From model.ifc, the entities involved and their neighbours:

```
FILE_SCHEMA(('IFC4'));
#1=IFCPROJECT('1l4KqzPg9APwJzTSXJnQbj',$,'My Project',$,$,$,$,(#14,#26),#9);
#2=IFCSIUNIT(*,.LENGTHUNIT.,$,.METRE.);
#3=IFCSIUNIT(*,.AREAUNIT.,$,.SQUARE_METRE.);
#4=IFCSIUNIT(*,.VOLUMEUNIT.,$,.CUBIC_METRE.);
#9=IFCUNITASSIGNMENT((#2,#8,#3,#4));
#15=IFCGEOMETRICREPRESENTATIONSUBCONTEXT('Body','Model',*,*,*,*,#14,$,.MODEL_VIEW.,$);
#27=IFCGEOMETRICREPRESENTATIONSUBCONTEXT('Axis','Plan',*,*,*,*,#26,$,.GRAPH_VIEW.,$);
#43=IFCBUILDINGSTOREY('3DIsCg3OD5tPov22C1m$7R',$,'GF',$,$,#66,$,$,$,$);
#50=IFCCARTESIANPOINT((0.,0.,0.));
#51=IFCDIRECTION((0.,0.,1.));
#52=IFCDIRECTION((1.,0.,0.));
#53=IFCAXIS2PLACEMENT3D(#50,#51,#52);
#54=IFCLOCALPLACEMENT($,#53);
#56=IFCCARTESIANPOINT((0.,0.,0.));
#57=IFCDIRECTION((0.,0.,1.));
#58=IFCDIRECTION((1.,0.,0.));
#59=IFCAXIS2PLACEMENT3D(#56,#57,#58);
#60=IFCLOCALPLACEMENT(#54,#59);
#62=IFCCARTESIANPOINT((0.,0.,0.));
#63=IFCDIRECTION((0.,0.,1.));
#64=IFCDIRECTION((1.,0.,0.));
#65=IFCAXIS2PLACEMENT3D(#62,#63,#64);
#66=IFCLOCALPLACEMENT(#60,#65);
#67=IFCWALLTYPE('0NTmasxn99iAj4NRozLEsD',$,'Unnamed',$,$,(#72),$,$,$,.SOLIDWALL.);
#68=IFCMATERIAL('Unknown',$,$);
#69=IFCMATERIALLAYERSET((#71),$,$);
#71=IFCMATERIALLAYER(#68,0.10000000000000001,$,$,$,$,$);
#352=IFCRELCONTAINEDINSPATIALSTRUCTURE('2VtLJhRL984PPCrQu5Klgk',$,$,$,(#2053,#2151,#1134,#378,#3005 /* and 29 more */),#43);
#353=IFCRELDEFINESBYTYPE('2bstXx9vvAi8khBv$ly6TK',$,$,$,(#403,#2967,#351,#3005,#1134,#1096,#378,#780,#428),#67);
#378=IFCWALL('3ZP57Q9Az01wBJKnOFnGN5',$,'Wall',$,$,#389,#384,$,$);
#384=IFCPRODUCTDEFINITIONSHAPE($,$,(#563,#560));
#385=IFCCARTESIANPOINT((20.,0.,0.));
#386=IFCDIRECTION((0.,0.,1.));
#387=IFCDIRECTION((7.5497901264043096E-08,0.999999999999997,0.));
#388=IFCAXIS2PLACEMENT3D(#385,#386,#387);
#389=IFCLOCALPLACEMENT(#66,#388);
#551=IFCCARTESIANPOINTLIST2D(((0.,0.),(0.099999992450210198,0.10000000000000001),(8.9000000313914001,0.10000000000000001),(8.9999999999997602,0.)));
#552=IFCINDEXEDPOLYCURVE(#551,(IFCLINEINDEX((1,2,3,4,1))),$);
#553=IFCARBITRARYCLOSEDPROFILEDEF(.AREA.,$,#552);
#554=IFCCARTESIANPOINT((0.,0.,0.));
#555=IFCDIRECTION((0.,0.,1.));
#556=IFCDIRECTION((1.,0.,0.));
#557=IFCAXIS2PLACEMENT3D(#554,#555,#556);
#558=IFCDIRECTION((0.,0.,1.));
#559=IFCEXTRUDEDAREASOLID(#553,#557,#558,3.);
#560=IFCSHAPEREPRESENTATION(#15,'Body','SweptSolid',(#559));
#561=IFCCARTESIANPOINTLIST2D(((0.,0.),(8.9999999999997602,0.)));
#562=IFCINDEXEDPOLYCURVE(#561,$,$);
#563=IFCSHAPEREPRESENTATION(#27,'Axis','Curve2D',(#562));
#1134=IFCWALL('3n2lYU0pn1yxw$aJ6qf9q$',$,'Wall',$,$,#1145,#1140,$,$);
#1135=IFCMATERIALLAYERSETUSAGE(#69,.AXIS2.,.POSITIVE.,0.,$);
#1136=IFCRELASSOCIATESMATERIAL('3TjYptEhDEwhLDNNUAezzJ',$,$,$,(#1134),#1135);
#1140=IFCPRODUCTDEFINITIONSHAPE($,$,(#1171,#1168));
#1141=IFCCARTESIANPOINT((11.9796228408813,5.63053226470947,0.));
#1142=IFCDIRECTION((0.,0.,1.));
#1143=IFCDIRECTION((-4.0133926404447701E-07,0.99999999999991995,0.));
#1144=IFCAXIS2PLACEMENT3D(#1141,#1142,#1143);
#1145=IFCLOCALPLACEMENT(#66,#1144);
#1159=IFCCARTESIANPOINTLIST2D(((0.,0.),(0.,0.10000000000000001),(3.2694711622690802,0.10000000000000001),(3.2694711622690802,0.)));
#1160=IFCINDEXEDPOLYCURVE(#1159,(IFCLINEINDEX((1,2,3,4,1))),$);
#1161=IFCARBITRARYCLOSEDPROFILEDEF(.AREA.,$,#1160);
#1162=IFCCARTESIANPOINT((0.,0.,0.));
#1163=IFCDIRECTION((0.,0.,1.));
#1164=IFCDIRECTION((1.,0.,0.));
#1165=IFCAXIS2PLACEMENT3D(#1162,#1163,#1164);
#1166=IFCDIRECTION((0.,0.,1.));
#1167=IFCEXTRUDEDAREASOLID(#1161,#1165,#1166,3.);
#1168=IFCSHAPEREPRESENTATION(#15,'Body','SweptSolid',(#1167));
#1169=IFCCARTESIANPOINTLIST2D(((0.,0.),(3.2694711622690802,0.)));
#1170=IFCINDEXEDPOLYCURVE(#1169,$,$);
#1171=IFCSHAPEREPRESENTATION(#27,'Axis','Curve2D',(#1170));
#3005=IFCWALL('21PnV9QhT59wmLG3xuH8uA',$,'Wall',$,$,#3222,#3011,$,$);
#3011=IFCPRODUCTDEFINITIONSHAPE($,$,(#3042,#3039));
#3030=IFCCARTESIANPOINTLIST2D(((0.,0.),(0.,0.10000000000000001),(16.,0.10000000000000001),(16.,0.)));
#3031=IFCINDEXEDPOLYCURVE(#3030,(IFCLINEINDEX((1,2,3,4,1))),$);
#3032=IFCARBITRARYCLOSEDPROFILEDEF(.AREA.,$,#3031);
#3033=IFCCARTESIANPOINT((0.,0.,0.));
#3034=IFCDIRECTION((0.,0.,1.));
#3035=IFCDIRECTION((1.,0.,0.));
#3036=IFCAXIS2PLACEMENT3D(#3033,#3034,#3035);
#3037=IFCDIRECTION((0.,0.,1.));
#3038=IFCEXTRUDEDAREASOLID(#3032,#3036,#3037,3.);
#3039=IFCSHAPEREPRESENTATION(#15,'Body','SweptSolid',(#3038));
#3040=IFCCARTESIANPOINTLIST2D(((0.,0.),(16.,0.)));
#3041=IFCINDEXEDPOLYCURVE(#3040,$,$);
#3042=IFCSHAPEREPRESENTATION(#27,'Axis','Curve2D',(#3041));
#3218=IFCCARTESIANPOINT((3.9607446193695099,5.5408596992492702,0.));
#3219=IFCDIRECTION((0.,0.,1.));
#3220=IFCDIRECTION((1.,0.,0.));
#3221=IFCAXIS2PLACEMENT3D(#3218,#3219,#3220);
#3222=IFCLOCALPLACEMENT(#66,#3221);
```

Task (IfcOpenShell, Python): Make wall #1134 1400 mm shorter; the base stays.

```python
import ifcopenshell
import ifcopenshell.geom
import ifcopenshell.util.representation
import ifcopenshell.util.shape
import ifcopenshell.util.unit

model = ifcopenshell.open("model.ifc")
unit_scale = ifcopenshell.util.unit.calculate_unit_scale(model)
settings = ifcopenshell.geom.settings()


def volume(element):
    """Net volume in cubic metres, openings subtracted."""
    shape = ifcopenshell.geom.create_shape(settings, element)
    return ifcopenshell.util.shape.get_volume(shape.geometry)


wall = model.by_id(1134)
before = volume(wall)

body = ifcopenshell.util.representation.get_representation(wall, "Model", "Body")
solid = body.Items[0]
old_height = solid.Depth
solid.Depth -= 1.4 / unit_scale
after = volume(wall)

print(f"height {old_height:g} -> {solid.Depth:g}, volume {before:.3f} -> {after:.3f} m3")

model.write("model_v2.ifc")
```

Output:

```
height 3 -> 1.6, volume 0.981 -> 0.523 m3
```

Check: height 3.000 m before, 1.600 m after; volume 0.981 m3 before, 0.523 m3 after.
